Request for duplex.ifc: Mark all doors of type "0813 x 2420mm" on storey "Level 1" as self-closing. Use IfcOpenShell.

First a look at what the model holds.

```python
import ifcopenshell
import ifcopenshell.util.element

model = ifcopenshell.open("duplex.ifc")
print(model.schema)
storey = next(s for s in model.by_type("IfcBuildingStorey") if s.Name == "Level 1")
doors = [e for e in ifcopenshell.util.element.get_decomposition(storey) if e.is_a("IfcDoor")]
seen = {}
for e in doors:
    element_type = ifcopenshell.util.element.get_type(e)
    key = (element_type.Name if element_type != e and element_type else None, ifcopenshell.util.element.get_pset(e, "Pset_DoorCommon", "SelfClosing"))
    seen[key] = seen.get(key, 0) + 1
for (name, value), count in sorted(seen.items(), key=str):
    print(count, "x", name, "|", value)
```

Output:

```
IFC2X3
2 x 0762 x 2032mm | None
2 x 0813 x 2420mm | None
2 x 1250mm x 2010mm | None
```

```python
import ifcopenshell
import ifcopenshell.api.pset
import ifcopenshell.util.element

model = ifcopenshell.open("duplex.ifc")

storey = next(s for s in model.by_type("IfcBuildingStorey") if s.Name == "Level 1")
doors = [e for e in ifcopenshell.util.element.get_decomposition(storey) if e.is_a("IfcDoor")]

count = 0
for e in doors:
    element_type = ifcopenshell.util.element.get_type(e)
    if element_type in (None, e) or element_type.Name != "0813 x 2420mm":
        continue
    # add_pset returns the element's existing set when there is one.
    pset = ifcopenshell.api.pset.add_pset(model, product=e, name="Pset_DoorCommon")
    ifcopenshell.api.pset.edit_pset(model, pset=pset, properties={"SelfClosing": True})
    count += 1

print(count, "doors updated")

model.write("duplex_rev.ifc")
```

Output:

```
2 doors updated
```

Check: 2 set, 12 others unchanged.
